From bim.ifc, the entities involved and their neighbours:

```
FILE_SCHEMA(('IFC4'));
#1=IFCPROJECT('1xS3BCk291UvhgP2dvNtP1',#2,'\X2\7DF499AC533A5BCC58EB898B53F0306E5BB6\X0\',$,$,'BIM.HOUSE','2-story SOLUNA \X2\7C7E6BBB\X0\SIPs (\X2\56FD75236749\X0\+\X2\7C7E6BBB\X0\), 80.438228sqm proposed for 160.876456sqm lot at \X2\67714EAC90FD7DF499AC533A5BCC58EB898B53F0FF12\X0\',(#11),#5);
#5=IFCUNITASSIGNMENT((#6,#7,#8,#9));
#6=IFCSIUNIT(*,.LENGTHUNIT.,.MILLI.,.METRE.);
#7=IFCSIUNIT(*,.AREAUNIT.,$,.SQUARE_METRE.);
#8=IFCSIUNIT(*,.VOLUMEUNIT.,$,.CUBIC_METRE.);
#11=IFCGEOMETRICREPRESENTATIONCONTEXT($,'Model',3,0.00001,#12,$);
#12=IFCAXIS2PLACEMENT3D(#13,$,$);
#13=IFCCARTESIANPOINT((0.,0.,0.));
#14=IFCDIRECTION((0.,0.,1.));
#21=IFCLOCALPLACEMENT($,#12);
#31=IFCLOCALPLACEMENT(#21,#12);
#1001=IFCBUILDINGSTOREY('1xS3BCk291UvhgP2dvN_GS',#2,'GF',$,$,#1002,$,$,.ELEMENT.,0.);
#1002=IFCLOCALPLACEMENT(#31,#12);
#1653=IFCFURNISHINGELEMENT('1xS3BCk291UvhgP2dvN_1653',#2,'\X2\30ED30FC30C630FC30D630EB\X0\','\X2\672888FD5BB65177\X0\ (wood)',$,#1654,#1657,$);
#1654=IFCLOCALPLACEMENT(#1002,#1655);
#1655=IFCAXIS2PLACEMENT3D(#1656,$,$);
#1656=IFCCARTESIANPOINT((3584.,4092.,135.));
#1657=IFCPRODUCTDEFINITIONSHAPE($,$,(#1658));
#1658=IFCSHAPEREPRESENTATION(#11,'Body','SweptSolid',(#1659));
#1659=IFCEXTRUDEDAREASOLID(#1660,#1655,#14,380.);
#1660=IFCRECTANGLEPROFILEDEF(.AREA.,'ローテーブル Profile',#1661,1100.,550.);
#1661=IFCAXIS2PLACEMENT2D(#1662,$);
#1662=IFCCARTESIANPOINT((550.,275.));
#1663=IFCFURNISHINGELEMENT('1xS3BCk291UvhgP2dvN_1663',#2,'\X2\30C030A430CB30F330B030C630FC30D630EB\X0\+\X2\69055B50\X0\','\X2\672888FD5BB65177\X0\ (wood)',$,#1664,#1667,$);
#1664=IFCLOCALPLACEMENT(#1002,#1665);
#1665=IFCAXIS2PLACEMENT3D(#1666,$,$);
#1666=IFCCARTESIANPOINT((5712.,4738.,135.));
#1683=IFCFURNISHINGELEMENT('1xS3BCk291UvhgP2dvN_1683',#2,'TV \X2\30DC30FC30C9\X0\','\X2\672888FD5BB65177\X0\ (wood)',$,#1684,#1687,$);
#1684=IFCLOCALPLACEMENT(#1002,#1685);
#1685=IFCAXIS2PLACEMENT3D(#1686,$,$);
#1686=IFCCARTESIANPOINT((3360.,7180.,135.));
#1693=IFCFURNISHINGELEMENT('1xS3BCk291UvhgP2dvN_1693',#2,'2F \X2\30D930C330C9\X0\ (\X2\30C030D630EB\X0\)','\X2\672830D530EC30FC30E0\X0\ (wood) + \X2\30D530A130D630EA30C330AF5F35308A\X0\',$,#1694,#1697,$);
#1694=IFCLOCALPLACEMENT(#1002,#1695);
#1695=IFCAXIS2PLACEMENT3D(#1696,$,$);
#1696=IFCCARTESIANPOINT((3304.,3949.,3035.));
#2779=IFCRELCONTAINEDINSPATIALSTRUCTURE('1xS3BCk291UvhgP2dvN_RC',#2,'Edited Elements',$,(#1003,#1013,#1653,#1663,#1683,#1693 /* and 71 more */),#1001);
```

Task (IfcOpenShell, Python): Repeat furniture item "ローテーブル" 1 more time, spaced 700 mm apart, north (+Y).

```python
import numpy as np
import ifcopenshell
import ifcopenshell.api.geometry
import ifcopenshell.api.root
import ifcopenshell.util.element
import ifcopenshell.util.placement
import ifcopenshell.util.unit

model = ifcopenshell.open("bim.ifc")
unit_scale = ifcopenshell.util.unit.calculate_unit_scale(model)


def reuse_history(source, copy):
    """copy_class also copies each property set's owner history, people and application; keep the originals."""
    for rel in copy.IsDefinedBy:
        if rel.is_a("IfcRelDefinesByProperties") and (history := rel.RelatingPropertyDefinition.OwnerHistory):
            rel.RelatingPropertyDefinition.OwnerHistory = source.OwnerHistory
            ifcopenshell.util.element.remove_deep2(model, history)


source = model.by_guid("1xS3BCk291UvhgP2dvN_1653")
base = ifcopenshell.util.placement.get_local_placement(source.ObjectPlacement)
step = np.array([0.0, 1.0, 0.0]) * 0.7 / unit_scale

for i in range(1, 2):
    copy = ifcopenshell.api.root.copy_class(model, product=source)
    copy.Representation = ifcopenshell.util.element.copy_deep(
        model, source.Representation, exclude=["IfcGeometricRepresentationContext", "IfcRepresentationMap"]
    )
    reuse_history(source, copy)
    matrix = base.copy()
    matrix[:3, 3] += i * step
    print("added at", matrix[:3, 3].round(3) + 0.0)
    ifcopenshell.api.geometry.edit_object_placement(model, product=copy, matrix=matrix, is_si=False)

model.write("bim_updated.ifc")
```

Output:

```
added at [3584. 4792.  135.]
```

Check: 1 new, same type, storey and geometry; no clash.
